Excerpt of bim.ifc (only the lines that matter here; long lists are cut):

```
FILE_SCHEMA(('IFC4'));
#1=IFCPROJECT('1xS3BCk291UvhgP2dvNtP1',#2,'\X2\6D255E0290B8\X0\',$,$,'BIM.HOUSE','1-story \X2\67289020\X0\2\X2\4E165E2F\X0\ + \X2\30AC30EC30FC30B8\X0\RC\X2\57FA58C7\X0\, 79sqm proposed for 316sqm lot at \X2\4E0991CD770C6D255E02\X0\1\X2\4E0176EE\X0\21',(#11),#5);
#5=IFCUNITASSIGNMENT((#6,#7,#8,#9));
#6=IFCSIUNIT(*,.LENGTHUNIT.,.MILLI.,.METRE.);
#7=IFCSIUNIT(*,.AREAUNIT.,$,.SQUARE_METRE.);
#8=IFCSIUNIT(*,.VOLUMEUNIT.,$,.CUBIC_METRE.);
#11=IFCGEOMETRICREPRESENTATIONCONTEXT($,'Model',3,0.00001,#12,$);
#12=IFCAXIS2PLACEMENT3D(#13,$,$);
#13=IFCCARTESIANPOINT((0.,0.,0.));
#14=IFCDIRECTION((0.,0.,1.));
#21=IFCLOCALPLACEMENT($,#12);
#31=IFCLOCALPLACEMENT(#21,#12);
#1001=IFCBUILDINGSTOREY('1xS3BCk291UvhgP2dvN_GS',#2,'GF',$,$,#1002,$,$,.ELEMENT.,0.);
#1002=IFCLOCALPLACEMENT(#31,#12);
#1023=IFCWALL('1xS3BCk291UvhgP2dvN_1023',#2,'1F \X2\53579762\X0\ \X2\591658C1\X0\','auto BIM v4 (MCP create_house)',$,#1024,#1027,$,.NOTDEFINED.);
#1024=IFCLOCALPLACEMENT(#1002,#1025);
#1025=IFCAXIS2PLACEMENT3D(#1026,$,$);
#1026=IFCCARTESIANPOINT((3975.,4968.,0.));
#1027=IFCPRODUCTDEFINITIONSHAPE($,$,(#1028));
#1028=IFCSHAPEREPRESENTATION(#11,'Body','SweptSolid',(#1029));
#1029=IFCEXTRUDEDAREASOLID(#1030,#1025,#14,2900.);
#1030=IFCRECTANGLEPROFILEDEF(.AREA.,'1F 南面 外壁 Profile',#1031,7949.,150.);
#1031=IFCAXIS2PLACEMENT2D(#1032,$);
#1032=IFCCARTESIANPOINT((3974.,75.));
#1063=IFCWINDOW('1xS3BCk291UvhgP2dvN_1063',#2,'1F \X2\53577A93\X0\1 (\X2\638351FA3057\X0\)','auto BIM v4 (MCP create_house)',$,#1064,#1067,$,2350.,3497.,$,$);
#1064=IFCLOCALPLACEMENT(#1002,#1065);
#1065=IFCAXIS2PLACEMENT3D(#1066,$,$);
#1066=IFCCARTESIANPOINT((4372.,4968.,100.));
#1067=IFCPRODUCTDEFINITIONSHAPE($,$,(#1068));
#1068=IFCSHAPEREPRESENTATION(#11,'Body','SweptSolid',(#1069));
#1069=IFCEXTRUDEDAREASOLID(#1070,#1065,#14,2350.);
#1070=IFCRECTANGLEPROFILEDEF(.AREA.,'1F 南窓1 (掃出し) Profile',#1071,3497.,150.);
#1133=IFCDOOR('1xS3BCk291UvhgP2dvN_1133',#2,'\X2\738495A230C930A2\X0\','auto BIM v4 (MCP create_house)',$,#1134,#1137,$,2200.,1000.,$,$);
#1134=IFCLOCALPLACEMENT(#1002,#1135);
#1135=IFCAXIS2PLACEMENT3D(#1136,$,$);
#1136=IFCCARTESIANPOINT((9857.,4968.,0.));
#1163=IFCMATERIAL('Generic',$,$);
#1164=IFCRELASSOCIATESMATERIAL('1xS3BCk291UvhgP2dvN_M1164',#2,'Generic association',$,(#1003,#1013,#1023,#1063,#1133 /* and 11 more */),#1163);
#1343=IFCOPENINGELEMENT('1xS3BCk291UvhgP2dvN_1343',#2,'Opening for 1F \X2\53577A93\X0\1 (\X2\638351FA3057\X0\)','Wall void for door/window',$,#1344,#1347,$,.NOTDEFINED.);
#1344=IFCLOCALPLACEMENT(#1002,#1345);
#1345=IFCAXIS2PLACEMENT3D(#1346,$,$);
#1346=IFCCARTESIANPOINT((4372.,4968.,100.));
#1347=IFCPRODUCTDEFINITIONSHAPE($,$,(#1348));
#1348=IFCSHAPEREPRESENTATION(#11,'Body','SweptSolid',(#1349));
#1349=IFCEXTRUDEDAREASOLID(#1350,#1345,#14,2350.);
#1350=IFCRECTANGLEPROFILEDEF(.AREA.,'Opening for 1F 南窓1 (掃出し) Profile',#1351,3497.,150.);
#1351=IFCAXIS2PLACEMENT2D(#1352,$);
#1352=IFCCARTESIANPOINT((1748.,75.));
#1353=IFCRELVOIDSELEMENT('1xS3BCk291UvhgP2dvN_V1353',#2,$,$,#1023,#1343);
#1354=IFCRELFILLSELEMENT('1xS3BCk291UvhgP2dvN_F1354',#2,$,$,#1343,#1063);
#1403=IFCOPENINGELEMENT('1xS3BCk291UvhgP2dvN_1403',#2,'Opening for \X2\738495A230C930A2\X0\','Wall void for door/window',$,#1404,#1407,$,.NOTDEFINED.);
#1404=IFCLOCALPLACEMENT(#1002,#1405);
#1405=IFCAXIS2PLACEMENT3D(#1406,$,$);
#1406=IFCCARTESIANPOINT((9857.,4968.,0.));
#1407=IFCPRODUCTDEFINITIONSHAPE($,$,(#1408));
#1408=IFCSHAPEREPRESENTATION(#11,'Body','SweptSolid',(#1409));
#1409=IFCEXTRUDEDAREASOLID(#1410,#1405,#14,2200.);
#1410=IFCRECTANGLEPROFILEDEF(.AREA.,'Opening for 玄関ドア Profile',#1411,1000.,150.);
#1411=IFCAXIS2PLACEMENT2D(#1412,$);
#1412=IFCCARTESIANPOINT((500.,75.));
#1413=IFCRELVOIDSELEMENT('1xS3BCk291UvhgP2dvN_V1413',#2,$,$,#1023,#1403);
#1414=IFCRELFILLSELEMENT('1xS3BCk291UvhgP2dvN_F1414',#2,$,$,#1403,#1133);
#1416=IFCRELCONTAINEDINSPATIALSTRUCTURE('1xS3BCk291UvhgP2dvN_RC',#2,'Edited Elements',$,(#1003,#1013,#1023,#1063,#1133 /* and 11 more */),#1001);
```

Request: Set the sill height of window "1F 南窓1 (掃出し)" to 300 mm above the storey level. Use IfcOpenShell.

```python
import numpy as np
import ifcopenshell
import ifcopenshell.api.geometry
import ifcopenshell.geom
import ifcopenshell.util.element
import ifcopenshell.util.placement
import ifcopenshell.util.shape
import ifcopenshell.util.unit

model = ifcopenshell.open("bim.ifc")
unit_scale = ifcopenshell.util.unit.calculate_unit_scale(model)

window = model.by_guid("1xS3BCk291UvhgP2dvN_1063")
opening = window.FillsVoids[0].RelatingOpeningElement
storey = ifcopenshell.util.element.get_container(window, ifc_class="IfcBuildingStorey")
level = ifcopenshell.util.placement.get_local_placement(storey.ObjectPlacement)[2, 3]

# The opening's origin need not be at the sill, so measure its lowest point.
shape = ifcopenshell.geom.create_shape(ifcopenshell.geom.settings(), opening)
bottom = ifcopenshell.util.shape.get_shape_bottom_elevation(shape, shape.geometry) / unit_scale
dz = level + 0.3 / unit_scale - bottom

shift = np.array([0.0, 0.0, dz])
# The window is not placed relative to its opening, so move both.
for product in (opening, window):
    matrix = ifcopenshell.util.placement.get_local_placement(product.ObjectPlacement)
    matrix[:3, 3] += shift
    ifcopenshell.api.geometry.edit_object_placement(model, product=product, matrix=matrix, is_si=False)

print(f"moved by {dz * unit_scale:+.3f} m")

model.write("bim_rev.ifc")
```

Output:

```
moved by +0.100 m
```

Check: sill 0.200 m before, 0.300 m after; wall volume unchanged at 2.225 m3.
